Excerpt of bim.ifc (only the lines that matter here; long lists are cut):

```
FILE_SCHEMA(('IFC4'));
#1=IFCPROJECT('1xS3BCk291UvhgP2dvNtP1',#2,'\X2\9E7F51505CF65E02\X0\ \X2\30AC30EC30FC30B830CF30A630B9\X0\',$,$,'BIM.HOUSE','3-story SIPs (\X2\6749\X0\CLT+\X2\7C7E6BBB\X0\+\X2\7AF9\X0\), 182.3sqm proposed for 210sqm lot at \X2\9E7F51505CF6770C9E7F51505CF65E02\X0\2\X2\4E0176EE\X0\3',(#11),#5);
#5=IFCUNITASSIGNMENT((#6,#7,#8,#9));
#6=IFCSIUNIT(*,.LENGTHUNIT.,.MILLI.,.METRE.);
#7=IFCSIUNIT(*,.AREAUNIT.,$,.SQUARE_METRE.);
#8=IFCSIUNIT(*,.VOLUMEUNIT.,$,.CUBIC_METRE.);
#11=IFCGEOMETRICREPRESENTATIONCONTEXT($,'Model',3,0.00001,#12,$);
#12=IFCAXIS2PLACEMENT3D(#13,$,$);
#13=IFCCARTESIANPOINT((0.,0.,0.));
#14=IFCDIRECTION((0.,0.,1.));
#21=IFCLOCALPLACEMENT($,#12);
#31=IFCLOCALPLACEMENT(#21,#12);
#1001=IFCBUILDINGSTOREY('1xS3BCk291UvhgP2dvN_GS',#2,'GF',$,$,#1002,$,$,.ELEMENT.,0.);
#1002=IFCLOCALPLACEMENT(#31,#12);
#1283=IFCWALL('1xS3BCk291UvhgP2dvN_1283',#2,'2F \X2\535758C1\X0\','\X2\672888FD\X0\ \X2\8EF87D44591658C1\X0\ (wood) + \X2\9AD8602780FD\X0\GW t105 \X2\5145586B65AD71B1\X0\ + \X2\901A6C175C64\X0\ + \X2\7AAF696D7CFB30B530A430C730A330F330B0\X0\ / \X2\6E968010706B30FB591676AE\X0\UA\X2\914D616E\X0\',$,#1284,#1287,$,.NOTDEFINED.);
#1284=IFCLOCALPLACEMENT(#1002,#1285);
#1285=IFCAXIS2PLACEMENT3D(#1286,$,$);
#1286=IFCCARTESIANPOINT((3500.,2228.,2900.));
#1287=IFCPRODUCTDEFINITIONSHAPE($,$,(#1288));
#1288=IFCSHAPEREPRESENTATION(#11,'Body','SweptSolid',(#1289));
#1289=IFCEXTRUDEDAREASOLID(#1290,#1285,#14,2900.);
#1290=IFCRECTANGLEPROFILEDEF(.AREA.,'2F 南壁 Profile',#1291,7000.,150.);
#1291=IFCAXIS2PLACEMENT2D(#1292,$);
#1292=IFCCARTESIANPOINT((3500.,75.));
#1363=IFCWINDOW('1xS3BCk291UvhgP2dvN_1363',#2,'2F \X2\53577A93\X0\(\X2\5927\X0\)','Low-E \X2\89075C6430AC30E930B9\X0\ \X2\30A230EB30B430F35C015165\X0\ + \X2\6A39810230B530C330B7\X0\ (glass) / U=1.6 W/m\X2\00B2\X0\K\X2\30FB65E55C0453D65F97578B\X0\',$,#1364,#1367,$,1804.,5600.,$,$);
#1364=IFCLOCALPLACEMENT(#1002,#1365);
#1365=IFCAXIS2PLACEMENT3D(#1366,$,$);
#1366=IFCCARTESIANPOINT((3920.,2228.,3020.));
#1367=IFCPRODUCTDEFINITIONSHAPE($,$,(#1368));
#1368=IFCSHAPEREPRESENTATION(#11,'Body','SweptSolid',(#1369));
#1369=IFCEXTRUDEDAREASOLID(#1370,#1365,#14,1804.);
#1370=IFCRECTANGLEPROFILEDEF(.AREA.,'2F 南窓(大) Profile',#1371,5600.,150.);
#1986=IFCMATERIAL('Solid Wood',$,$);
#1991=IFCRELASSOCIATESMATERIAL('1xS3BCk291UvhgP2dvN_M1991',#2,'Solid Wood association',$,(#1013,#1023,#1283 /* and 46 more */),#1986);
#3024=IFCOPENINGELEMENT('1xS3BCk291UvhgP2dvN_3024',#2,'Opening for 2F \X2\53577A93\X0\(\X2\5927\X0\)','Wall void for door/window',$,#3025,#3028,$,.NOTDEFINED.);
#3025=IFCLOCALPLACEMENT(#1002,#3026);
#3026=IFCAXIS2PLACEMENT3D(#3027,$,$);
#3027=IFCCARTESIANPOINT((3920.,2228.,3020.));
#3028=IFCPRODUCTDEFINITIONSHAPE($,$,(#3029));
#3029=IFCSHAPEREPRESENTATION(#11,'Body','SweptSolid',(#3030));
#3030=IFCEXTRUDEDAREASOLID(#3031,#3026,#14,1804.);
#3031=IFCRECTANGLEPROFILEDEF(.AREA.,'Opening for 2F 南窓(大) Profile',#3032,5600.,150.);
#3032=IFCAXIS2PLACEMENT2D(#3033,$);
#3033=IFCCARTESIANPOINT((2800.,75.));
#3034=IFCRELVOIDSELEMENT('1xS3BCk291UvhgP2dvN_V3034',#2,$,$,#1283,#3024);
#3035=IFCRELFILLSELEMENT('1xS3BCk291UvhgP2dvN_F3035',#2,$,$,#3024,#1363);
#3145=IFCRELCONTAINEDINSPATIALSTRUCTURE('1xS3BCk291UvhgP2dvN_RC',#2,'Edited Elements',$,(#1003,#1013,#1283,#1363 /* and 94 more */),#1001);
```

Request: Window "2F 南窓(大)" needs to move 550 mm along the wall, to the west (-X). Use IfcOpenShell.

```python
import ifcopenshell
import ifcopenshell.api.geometry
import ifcopenshell.util.placement

model = ifcopenshell.open("bim.ifc")

window = model.by_id(1363)
opening = window.FillsVoids[0].RelatingOpeningElement
wall = opening.VoidsElements[0].RelatingBuildingElement

wall_matrix = ifcopenshell.util.placement.get_local_placement(wall.ObjectPlacement)
shift = wall_matrix[:3, 0] * -550.0
before = ifcopenshell.util.placement.get_local_placement(window.ObjectPlacement)[:3, 3].copy()

# The window is not placed relative to its opening, so move both.
for product in (opening, window):
    matrix = ifcopenshell.util.placement.get_local_placement(product.ObjectPlacement)
    matrix[:3, 3] += shift
    ifcopenshell.api.geometry.edit_object_placement(model, product=product, matrix=matrix, is_si=False)

after = ifcopenshell.util.placement.get_local_placement(window.ObjectPlacement)[:3, 3]
print("window moved by", (after - before).round(3) + 0.0)

model.write("bim_edited.ifc")
```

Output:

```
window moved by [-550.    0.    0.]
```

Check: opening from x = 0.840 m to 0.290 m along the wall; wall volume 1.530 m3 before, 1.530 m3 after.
